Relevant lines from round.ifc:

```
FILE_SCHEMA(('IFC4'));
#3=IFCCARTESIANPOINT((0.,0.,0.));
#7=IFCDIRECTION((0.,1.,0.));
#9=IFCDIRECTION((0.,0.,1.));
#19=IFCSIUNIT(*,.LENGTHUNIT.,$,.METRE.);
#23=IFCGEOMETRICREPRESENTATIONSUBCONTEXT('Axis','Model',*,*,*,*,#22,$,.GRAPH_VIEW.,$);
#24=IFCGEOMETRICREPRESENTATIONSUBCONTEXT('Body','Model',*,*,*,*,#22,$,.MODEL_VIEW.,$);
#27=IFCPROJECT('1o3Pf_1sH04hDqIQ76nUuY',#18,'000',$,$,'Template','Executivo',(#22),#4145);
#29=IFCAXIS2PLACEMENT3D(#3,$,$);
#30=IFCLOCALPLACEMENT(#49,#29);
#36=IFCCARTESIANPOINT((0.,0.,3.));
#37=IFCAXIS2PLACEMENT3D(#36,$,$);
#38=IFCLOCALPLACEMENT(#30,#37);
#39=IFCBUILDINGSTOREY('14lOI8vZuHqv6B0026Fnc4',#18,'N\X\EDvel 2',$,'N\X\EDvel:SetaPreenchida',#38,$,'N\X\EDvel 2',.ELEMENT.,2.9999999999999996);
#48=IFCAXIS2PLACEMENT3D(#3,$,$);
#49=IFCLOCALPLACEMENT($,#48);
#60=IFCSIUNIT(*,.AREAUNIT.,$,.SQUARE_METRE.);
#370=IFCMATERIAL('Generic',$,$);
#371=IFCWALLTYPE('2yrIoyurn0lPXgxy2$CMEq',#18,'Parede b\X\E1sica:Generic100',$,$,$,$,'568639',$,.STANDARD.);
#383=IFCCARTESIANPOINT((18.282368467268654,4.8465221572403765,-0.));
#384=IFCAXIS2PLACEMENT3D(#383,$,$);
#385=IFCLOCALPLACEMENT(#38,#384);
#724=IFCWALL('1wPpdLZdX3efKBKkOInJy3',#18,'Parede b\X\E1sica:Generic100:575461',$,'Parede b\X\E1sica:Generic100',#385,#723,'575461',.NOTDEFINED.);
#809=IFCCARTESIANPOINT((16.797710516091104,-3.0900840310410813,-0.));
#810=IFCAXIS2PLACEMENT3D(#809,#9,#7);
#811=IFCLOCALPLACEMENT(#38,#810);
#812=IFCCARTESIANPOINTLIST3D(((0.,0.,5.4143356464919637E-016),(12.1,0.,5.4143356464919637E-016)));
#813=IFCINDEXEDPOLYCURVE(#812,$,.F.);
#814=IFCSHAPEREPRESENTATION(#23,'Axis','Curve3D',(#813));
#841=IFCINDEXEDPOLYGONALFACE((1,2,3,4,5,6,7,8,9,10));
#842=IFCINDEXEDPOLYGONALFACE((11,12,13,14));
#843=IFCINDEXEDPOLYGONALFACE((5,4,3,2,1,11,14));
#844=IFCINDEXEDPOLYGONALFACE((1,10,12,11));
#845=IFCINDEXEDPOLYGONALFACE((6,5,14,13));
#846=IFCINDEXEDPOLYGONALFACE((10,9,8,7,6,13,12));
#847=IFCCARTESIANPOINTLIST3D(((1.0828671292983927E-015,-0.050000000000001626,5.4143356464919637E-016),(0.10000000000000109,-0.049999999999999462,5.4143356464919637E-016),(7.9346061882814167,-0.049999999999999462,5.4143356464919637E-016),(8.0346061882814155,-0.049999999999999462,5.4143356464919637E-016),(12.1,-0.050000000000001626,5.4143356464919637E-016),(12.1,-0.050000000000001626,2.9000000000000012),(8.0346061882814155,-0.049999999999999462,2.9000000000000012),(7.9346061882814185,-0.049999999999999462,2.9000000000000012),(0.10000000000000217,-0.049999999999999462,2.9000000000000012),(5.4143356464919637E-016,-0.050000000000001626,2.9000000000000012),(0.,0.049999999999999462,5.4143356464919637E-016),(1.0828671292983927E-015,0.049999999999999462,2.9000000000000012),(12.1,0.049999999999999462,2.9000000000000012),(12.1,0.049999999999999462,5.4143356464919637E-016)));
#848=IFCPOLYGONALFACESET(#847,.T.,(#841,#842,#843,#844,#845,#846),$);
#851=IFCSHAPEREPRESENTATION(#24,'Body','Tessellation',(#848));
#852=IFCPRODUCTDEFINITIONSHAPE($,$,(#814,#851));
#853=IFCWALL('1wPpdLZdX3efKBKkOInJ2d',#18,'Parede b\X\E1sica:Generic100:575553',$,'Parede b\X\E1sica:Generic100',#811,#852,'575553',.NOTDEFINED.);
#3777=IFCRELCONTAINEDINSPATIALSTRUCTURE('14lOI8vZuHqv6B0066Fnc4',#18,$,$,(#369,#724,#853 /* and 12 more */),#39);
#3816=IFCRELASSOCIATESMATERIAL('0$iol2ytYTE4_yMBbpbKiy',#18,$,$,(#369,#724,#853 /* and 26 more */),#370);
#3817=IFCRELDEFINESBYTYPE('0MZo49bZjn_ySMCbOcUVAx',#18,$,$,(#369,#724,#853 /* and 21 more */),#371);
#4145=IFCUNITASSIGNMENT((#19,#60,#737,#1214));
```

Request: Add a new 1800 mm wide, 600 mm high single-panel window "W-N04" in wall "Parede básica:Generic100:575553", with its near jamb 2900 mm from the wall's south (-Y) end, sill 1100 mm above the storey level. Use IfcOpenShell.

```python
import numpy as np
import ifcopenshell
import ifcopenshell.api.feature
import ifcopenshell.api.geometry
import ifcopenshell.api.root
import ifcopenshell.api.spatial
import ifcopenshell.geom
import ifcopenshell.util.element
import ifcopenshell.util.placement
import ifcopenshell.util.representation
import ifcopenshell.util.shape
import ifcopenshell.util.unit

model = ifcopenshell.open("round.ifc")
unit_scale = ifcopenshell.util.unit.calculate_unit_scale(model)
settings = ifcopenshell.geom.settings()


def volume(element):
    """Net volume in cubic metres, openings subtracted."""
    shape = ifcopenshell.geom.create_shape(settings, element)
    return ifcopenshell.util.shape.get_volume(shape.geometry)


wall = model.by_id(853)
storey = ifcopenshell.util.element.get_container(wall, ifc_class="IfcBuildingStorey")
context = ifcopenshell.util.representation.get_context(model, "Model", "Body", "MODEL_VIEW")
before = volume(wall)

width, height, from_end, sill = 1.8, 0.6, 2.9, 1.1  # metres

# The wall runs along its own X axis, and the end named is its -X end.
wall_shape = ifcopenshell.geom.create_shape(settings, wall)
x, y, z = ifcopenshell.util.shape.get_vertices(wall_shape.geometry).T
start = x.min() + from_end
face, thickness = float(y.min()), float(y.max() - y.min())
wall_matrix = ifcopenshell.util.placement.get_local_placement(wall.ObjectPlacement)
level = ifcopenshell.util.placement.get_local_placement(storey.ObjectPlacement)[2, 3]


def in_wall(x, y):
    """Placement at x, y metres in the wall's axes, at sill height."""
    matrix = wall_matrix.copy()
    matrix[:, 3] = wall_matrix @ np.array([x / unit_scale, y / unit_scale, 0.0, 1.0])
    matrix[2, 3] = level + sill / unit_scale
    return matrix


# Opening: a box that overshoots both wall faces by 50 mm.
opening = ifcopenshell.api.root.create_entity(model, ifc_class="IfcOpeningElement", predefined_type="OPENING")
box = ifcopenshell.api.geometry.add_wall_representation(
    model, context=context, length=width, height=height, thickness=thickness + 0.1
)
ifcopenshell.api.geometry.assign_representation(model, product=opening, representation=box)
ifcopenshell.api.geometry.edit_object_placement(model, product=opening, matrix=in_wall(start, face - 0.05), is_si=False)
ifcopenshell.api.feature.add_feature(model, feature=opening, element=wall)

window = ifcopenshell.api.root.create_entity(model, ifc_class="IfcWindow", name="W-N04", predefined_type="WINDOW")
window.OverallWidth, window.OverallHeight = width / unit_scale, height / unit_scale
window.PartitioningType = "SINGLE_PANEL"
body = ifcopenshell.api.geometry.add_window_representation(
    model,
    context=context,
    overall_width=window.OverallWidth,
    overall_height=window.OverallHeight,
    partition_type="SINGLE_PANEL",
)
ifcopenshell.api.geometry.assign_representation(model, product=window, representation=body)
ifcopenshell.api.spatial.assign_container(model, products=[window], relating_structure=storey)
ifcopenshell.api.feature.add_filling(model, opening=opening, element=window)

# Centre the window in the wall's thickness.
ifcopenshell.api.geometry.edit_object_placement(model, product=window, matrix=in_wall(start, face), is_si=False)
window_shape = ifcopenshell.geom.create_shape(settings, window)
depth = ifcopenshell.util.shape.get_vertices(window_shape.geometry)[:, 1]
offset = face + thickness / 2 - (depth.min() + depth.max()) / 2
ifcopenshell.api.geometry.edit_object_placement(model, product=window, matrix=in_wall(start, offset), is_si=False)

after = volume(wall)

print(f"wall volume {before:.3f} -> {after:.3f} m3")

model.write("round_rev.ifc")
```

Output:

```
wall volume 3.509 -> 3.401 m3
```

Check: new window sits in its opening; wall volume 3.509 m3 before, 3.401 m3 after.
